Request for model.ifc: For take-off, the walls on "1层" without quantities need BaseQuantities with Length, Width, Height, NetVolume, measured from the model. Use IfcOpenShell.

First a look at what the model holds.

```python
import ifcopenshell
import ifcopenshell.util.element
import ifcopenshell.util.unit

model = ifcopenshell.open("model.ifc")
print(model.schema)
for unit_type in ("LENGTHUNIT", "AREAUNIT", "VOLUMEUNIT"):
    print(unit_type, ifcopenshell.util.unit.calculate_unit_scale(model, unit_type))
storey = next(s for s in model.by_type("IfcBuildingStorey") if s.Name == "1层")
walls = [e for e in ifcopenshell.util.element.get_decomposition(storey) if e.is_a("IfcWall")]
for e in sorted(walls, key=lambda e: e.id()):
    print(e.id(), e.is_a(), e.Name, list(ifcopenshell.util.element.get_psets(e, qtos_only=True)), sep=" | ")
```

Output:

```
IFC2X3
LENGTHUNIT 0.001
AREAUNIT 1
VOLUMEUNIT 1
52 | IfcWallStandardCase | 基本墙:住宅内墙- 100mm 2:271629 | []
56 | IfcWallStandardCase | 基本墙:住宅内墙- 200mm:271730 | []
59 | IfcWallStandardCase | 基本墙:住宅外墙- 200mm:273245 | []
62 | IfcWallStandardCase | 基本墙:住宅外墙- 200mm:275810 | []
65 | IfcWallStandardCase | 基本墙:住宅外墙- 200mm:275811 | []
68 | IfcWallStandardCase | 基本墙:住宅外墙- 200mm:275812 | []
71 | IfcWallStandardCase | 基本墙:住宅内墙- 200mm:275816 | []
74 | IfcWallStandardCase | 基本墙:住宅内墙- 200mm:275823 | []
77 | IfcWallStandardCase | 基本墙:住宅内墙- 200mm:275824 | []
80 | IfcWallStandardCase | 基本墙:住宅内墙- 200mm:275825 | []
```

```python
import ifcopenshell
import ifcopenshell.api.pset
import ifcopenshell.geom
import ifcopenshell.util.element
import ifcopenshell.util.shape
import ifcopenshell.util.unit

model = ifcopenshell.open("model.ifc")
unit_scale = ifcopenshell.util.unit.calculate_unit_scale(model)
volume_scale = ifcopenshell.util.unit.calculate_unit_scale(model, "VOLUMEUNIT")
settings = ifcopenshell.geom.settings()

storey = next(s for s in model.by_type("IfcBuildingStorey") if s.Name == "1层")
walls = [e for e in ifcopenshell.util.element.get_decomposition(storey) if e.is_a("IfcWall")]

for e in sorted(walls, key=lambda e: e.id()):
    if ifcopenshell.util.element.get_psets(e, qtos_only=True, should_inherit=False):
        continue
    # Geometry comes back in metres, in the element's own axes.
    shape = ifcopenshell.geom.create_shape(settings, e)
    values = {
        "Length": ifcopenshell.util.shape.get_x(shape.geometry) / unit_scale,
        "Width": ifcopenshell.util.shape.get_y(shape.geometry) / unit_scale,
        "Height": ifcopenshell.util.shape.get_z(shape.geometry) / unit_scale,
        "NetVolume": ifcopenshell.util.shape.get_volume(shape.geometry) / volume_scale,
    }
    qto = ifcopenshell.api.pset.add_qto(model, product=e, name="BaseQuantities")
    ifcopenshell.api.pset.edit_qto(model, qto=qto, properties=values)
    print(e.id(), {k: round(v, 3) for k, v in values.items()})

model.write("model_v2.ifc")
```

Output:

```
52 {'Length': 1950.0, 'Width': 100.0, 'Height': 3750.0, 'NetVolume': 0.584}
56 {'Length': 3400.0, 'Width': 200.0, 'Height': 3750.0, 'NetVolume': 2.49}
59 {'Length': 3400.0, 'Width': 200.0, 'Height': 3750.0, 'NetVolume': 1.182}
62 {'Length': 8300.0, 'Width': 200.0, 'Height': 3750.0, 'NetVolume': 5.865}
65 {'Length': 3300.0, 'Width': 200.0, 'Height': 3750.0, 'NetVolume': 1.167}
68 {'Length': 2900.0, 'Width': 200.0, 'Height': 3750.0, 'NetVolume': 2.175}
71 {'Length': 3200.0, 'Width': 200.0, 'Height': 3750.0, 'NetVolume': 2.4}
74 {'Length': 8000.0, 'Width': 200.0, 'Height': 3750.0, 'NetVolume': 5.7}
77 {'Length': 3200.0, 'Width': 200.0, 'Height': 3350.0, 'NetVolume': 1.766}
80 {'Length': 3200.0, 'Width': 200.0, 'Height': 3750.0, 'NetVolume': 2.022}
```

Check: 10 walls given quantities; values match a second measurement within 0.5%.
